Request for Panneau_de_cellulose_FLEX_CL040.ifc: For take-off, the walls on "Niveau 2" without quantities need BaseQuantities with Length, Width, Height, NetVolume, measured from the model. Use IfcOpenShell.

First a look at what the model holds.

```python
import ifcopenshell
import ifcopenshell.util.element
import ifcopenshell.util.unit

model = ifcopenshell.open("Panneau_de_cellulose_FLEX_CL040.ifc")
print(model.schema)
for unit_type in ("LENGTHUNIT", "AREAUNIT", "VOLUMEUNIT"):
    print(unit_type, ifcopenshell.util.unit.calculate_unit_scale(model, unit_type))
storey = next(s for s in model.by_type("IfcBuildingStorey") if s.Name == "Niveau 2")
walls = [e for e in ifcopenshell.util.element.get_decomposition(storey) if e.is_a("IfcWall")]
for e in sorted(walls, key=lambda e: e.id()):
    print(e.id(), e.is_a(), e.Name, list(ifcopenshell.util.element.get_psets(e, qtos_only=True)), sep=" | ")
```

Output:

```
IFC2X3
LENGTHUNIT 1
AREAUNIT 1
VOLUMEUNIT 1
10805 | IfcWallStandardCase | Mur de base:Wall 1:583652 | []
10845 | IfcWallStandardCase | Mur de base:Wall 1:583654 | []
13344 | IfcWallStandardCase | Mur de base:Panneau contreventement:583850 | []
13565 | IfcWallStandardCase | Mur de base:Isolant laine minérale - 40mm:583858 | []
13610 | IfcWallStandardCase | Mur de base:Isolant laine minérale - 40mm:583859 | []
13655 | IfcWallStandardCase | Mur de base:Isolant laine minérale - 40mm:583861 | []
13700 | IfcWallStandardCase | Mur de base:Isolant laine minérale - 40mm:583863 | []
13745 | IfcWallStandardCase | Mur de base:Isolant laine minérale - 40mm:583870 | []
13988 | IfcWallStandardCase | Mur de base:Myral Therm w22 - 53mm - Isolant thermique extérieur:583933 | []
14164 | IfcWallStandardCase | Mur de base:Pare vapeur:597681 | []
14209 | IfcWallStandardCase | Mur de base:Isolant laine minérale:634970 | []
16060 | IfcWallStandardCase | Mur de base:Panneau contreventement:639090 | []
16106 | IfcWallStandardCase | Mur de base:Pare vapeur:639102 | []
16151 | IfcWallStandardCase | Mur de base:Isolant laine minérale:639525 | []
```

```python
import ifcopenshell
import ifcopenshell.api.pset
import ifcopenshell.geom
import ifcopenshell.util.element
import ifcopenshell.util.shape
import ifcopenshell.util.unit

model = ifcopenshell.open("Panneau_de_cellulose_FLEX_CL040.ifc")
unit_scale = ifcopenshell.util.unit.calculate_unit_scale(model)
volume_scale = ifcopenshell.util.unit.calculate_unit_scale(model, "VOLUMEUNIT")
settings = ifcopenshell.geom.settings()

storey = next(s for s in model.by_type("IfcBuildingStorey") if s.Name == "Niveau 2")
walls = [e for e in ifcopenshell.util.element.get_decomposition(storey) if e.is_a("IfcWall")]

for e in sorted(walls, key=lambda e: e.id()):
    if ifcopenshell.util.element.get_psets(e, qtos_only=True, should_inherit=False):
        continue
    # Geometry comes back in metres, in the element's own axes.
    shape = ifcopenshell.geom.create_shape(settings, e)
    values = {
        "Length": ifcopenshell.util.shape.get_x(shape.geometry) / unit_scale,
        "Width": ifcopenshell.util.shape.get_y(shape.geometry) / unit_scale,
        "Height": ifcopenshell.util.shape.get_z(shape.geometry) / unit_scale,
        "NetVolume": ifcopenshell.util.shape.get_volume(shape.geometry) / volume_scale,
    }
    qto = ifcopenshell.api.pset.add_qto(model, product=e, name="BaseQuantities")
    ifcopenshell.api.pset.edit_qto(model, qto=qto, properties=values)
    print(e.id(), {k: round(v, 3) for k, v in values.items()})

model.write("Panneau_de_cellulose_FLEX_CL040_edited.ifc")
```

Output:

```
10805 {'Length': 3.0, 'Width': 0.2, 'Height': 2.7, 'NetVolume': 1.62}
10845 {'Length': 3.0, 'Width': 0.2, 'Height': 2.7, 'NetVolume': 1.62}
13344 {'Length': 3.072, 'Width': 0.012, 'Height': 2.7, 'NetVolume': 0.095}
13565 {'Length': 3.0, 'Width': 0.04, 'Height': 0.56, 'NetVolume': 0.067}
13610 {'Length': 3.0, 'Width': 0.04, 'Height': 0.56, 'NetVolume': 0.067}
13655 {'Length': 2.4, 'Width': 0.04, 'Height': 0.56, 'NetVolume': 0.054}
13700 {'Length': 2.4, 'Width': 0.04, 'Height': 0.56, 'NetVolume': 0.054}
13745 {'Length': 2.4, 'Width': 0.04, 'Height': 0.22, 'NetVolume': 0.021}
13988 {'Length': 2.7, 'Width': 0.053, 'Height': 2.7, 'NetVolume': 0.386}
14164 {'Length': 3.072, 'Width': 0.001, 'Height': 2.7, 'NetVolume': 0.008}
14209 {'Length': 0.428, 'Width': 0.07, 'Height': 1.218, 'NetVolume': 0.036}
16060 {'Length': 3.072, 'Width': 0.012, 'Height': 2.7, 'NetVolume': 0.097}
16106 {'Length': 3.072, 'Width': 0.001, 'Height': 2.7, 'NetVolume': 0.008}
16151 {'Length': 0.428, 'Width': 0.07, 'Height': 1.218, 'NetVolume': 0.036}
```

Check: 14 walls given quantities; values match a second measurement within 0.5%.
